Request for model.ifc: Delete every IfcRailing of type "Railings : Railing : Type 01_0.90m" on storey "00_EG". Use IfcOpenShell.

First a look at what the model holds.

```python
import ifcopenshell
import ifcopenshell.util.element

model = ifcopenshell.open("model.ifc")
print(model.schema)
storey = next(s for s in model.by_type("IfcBuildingStorey") if s.Name == "00_EG")
railings = [e for e in ifcopenshell.util.element.get_decomposition(storey) if e.is_a("IfcRailing")]
seen = {}
for e in railings:
    element_type = ifcopenshell.util.element.get_type(e)
    name = element_type.Name if element_type not in (None, e) else None
    seen[name] = seen.get(name, 0) + 1
for name, count in sorted(seen.items(), key=str):
    print(count, "x", name)
```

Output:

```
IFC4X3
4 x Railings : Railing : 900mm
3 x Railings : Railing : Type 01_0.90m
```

```python
import ifcopenshell
import ifcopenshell.api.root
import ifcopenshell.util.element

model = ifcopenshell.open("model.ifc")

storey = next(s for s in model.by_type("IfcBuildingStorey") if s.Name == "00_EG")
railings = [e for e in ifcopenshell.util.element.get_decomposition(storey) if e.is_a("IfcRailing")]
targets = [e for e in railings if (t := ifcopenshell.util.element.get_type(e)) not in (None, e) and t.Name == "Railings : Railing : Type 01_0.90m"]

for e in targets:
    ifcopenshell.api.root.remove_product(model, product=e)
print(len(targets), "removed")

model.write("model_v2.ifc")
```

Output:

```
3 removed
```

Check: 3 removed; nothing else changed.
